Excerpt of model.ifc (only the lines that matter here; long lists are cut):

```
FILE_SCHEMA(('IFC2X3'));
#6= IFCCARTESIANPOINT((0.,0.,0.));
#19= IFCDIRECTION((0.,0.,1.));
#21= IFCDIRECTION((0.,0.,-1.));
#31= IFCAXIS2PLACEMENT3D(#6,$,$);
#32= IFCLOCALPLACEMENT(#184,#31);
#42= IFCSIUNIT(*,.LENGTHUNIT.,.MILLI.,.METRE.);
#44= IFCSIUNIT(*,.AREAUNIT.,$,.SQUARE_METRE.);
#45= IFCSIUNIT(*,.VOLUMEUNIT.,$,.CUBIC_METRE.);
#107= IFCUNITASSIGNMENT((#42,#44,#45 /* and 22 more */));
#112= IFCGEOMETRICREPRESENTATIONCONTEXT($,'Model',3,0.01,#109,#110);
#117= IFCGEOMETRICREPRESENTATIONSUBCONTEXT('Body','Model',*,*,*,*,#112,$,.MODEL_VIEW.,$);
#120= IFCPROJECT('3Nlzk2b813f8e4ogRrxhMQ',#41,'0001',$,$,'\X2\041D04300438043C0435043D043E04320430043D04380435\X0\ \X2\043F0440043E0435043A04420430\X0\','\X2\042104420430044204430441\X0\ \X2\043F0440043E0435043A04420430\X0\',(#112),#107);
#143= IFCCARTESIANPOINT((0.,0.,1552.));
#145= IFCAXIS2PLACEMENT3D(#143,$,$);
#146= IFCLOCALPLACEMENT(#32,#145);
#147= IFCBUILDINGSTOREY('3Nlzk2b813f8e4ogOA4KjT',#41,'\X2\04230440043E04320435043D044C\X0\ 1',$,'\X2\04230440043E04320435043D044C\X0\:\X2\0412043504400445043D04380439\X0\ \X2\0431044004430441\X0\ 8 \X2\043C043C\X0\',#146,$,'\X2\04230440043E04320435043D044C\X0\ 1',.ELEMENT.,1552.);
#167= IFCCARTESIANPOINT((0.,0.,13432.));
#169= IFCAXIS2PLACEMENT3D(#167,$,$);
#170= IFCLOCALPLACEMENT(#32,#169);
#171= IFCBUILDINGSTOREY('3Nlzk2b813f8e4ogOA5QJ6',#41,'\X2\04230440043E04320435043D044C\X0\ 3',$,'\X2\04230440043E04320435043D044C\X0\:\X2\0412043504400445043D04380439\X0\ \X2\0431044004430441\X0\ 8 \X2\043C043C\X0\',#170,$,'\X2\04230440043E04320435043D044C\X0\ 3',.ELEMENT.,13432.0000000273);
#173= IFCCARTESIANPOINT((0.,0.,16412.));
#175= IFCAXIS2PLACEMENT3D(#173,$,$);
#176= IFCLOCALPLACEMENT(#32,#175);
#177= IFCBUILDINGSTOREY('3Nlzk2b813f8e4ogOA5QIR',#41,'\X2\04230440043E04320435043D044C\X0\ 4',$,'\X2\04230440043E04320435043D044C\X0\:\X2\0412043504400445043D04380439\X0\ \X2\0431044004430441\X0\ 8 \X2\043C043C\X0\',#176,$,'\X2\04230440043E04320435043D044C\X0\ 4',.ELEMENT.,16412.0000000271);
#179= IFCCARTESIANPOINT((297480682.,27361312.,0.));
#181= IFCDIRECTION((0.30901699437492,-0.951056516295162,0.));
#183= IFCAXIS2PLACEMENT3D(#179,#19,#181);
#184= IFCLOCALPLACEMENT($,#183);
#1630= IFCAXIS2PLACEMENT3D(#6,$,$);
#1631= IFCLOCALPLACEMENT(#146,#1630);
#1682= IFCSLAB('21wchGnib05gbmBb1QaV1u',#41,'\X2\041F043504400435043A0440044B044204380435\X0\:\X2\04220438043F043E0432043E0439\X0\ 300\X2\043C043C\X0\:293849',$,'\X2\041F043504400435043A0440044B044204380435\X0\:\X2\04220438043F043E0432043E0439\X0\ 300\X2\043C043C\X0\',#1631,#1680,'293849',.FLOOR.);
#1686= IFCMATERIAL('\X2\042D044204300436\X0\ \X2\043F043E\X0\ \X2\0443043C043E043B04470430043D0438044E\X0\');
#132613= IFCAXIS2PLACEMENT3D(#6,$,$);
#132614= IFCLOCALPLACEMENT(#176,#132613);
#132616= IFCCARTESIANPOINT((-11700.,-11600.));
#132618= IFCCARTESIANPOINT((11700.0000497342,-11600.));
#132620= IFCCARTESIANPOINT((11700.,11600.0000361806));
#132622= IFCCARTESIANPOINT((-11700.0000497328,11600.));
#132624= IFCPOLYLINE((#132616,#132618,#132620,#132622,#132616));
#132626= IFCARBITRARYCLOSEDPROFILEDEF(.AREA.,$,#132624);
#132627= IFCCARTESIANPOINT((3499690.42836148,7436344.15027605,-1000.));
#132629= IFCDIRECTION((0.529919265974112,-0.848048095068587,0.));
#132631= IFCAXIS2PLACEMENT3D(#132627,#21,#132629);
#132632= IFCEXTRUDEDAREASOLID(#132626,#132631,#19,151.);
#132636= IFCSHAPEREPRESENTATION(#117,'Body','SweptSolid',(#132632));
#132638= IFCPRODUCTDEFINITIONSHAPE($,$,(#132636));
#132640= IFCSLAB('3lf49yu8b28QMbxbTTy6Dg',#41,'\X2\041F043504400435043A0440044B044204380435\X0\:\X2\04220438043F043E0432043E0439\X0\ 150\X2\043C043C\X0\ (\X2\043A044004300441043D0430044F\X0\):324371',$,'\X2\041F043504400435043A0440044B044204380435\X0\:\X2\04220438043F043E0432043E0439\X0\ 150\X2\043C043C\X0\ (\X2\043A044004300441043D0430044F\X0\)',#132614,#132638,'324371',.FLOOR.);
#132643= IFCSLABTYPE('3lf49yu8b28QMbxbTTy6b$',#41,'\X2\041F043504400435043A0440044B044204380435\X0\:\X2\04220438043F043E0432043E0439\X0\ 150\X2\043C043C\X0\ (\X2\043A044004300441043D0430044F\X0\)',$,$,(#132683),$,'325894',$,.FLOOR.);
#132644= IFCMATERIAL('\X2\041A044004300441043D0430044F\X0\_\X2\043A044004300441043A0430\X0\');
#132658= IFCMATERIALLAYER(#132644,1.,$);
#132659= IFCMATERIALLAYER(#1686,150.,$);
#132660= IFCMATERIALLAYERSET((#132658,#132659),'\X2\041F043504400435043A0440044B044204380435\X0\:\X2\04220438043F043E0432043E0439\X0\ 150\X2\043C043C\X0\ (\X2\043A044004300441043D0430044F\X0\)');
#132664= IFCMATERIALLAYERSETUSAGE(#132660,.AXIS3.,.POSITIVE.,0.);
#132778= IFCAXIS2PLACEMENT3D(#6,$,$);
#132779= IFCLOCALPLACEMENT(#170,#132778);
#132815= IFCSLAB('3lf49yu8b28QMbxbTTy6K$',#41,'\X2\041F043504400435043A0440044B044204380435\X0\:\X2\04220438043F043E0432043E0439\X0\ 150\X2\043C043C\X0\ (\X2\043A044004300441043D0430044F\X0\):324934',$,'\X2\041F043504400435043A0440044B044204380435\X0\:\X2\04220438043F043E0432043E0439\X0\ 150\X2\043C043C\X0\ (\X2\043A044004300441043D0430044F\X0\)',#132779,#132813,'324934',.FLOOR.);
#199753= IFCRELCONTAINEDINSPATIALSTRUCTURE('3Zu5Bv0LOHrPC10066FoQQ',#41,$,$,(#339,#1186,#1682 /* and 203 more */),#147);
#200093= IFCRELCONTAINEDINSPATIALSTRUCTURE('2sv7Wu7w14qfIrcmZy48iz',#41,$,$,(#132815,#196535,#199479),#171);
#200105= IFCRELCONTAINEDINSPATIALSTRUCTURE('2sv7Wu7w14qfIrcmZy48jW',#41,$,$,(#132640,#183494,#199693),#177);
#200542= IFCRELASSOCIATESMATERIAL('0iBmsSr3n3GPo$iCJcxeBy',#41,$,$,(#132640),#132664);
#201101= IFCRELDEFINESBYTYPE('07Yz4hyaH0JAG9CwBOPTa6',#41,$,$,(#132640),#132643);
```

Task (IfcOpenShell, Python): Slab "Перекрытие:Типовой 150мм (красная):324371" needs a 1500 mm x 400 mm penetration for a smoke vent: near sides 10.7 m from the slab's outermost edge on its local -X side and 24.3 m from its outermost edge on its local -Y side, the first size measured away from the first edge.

```python
import numpy as np
import ifcopenshell
import ifcopenshell.api.feature
import ifcopenshell.api.geometry
import ifcopenshell.api.root
import ifcopenshell.geom
import ifcopenshell.util.placement
import ifcopenshell.util.representation
import ifcopenshell.util.shape
import ifcopenshell.util.unit

model = ifcopenshell.open("model.ifc")
unit_scale = ifcopenshell.util.unit.calculate_unit_scale(model)
settings = ifcopenshell.geom.settings()


def volume(element):
    """Net volume in cubic metres, openings subtracted."""
    shape = ifcopenshell.geom.create_shape(settings, element)
    return ifcopenshell.util.shape.get_volume(shape.geometry)


slab = model.by_id(132640)
before = volume(slab)

# Extent in the slab's own axes, in metres. The edges named are its -X and -Y sides.
slab_shape = ifcopenshell.geom.create_shape(settings, slab)
vertices = ifcopenshell.util.shape.get_vertices(slab_shape.geometry)
x_min, y_min, bottom = vertices.min(axis=0)
top = vertices[:, 2].max()

opening = ifcopenshell.api.root.create_entity(model, ifc_class="IfcOpeningElement", name="Smoke vent opening")
context = ifcopenshell.util.representation.get_context(model, "Model", "Body", "MODEL_VIEW")
width, depth = 1.5, 0.4
outline = [(0.0, 0.0), (width, 0.0), (width, depth), (0.0, depth), (0.0, 0.0)]
# Overshoot both faces by 50 mm so the cut is clean.
shape = ifcopenshell.api.geometry.add_slab_representation(
    model, context=context, depth=top - bottom + 0.1, polyline=outline
)
ifcopenshell.api.geometry.assign_representation(model, product=opening, representation=shape)

matrix = ifcopenshell.util.placement.get_local_placement(slab.ObjectPlacement)
matrix[:, 3] = matrix @ np.append(np.array([x_min + 10.7, y_min + 24.3, bottom - 0.05]) / unit_scale, 1.0)
ifcopenshell.api.geometry.edit_object_placement(model, product=opening, matrix=matrix, is_si=False)
ifcopenshell.api.feature.add_feature(model, feature=opening, element=slab)

after = volume(slab)

print(f"slab volume {before:.3f} -> {after:.3f} m3")

model.write("model_updated.ifc")
```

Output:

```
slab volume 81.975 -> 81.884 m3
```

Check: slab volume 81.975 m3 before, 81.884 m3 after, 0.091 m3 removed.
